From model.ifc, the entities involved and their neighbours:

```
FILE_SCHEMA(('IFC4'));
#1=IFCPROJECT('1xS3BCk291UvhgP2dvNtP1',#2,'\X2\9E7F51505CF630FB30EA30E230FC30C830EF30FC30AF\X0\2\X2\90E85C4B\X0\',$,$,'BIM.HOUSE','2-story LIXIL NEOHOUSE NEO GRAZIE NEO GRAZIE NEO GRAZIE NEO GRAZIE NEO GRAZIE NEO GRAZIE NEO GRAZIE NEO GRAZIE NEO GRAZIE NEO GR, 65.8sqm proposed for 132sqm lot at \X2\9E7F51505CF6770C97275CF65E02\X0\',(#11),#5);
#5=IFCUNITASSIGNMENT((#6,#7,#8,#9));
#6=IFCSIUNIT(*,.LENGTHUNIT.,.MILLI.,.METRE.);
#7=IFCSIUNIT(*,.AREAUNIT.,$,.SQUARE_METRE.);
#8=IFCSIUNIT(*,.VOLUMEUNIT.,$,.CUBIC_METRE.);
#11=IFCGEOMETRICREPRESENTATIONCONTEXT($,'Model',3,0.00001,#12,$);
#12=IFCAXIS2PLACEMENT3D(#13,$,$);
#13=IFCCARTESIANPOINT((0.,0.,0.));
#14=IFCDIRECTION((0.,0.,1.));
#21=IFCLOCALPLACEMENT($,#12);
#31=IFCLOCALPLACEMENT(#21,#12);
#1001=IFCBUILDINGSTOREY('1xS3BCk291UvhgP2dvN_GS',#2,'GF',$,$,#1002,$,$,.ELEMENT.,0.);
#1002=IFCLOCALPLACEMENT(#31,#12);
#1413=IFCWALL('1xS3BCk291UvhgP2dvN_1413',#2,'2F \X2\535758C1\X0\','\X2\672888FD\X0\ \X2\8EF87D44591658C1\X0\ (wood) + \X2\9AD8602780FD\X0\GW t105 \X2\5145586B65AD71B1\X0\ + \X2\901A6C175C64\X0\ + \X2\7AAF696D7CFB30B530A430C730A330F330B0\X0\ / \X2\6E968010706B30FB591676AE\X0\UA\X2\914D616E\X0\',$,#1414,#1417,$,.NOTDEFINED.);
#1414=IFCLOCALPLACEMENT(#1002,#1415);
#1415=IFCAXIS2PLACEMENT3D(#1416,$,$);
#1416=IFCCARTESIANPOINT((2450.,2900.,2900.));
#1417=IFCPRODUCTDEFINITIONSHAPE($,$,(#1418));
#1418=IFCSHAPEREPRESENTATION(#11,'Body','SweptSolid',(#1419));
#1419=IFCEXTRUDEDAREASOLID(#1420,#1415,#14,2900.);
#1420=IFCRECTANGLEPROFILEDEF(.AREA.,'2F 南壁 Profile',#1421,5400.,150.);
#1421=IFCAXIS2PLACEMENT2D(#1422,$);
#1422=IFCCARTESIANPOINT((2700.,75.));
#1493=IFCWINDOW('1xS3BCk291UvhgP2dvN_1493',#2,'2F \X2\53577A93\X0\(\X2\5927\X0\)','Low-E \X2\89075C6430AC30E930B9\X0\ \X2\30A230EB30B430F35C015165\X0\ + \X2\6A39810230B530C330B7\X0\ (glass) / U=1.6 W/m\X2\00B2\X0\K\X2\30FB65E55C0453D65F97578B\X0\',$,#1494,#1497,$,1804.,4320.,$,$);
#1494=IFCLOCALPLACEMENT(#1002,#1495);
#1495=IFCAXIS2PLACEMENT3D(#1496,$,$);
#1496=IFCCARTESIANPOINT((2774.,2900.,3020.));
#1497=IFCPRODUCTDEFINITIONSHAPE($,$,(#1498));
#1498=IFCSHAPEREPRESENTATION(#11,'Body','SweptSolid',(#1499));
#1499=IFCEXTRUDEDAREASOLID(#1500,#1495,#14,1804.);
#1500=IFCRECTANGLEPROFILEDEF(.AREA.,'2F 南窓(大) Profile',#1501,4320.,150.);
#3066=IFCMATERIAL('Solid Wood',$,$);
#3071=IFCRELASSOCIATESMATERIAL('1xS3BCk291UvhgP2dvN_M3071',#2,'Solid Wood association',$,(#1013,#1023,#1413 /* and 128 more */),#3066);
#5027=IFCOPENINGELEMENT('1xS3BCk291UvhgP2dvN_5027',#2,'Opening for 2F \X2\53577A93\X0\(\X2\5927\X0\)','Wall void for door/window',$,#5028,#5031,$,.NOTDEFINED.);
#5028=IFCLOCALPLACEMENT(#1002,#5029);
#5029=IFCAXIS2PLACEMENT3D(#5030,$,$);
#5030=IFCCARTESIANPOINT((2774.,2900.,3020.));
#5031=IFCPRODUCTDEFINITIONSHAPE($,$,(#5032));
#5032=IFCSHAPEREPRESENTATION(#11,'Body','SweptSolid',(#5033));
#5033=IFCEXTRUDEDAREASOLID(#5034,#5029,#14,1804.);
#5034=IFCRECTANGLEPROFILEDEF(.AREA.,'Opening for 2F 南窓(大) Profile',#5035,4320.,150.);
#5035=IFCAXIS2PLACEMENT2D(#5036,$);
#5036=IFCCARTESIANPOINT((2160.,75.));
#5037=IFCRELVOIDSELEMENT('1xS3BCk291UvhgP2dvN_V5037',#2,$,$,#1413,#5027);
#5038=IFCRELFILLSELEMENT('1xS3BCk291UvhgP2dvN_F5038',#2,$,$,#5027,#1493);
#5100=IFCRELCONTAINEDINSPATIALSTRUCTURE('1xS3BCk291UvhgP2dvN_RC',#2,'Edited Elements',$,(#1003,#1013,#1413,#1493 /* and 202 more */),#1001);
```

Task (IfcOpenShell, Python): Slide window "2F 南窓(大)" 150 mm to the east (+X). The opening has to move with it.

```python
import ifcopenshell
import ifcopenshell.api.geometry
import ifcopenshell.util.placement
import ifcopenshell.util.unit

model = ifcopenshell.open("model.ifc")
unit_scale = ifcopenshell.util.unit.calculate_unit_scale(model)

window = model.by_id(1493)
opening = window.FillsVoids[0].RelatingOpeningElement
wall = opening.VoidsElements[0].RelatingBuildingElement

wall_matrix = ifcopenshell.util.placement.get_local_placement(wall.ObjectPlacement)
shift = wall_matrix[:3, 0] * 0.15 / unit_scale
before = ifcopenshell.util.placement.get_local_placement(window.ObjectPlacement)[:3, 3].copy()

# The window is not placed relative to its opening, so move both.
for product in (opening, window):
    matrix = ifcopenshell.util.placement.get_local_placement(product.ObjectPlacement)
    matrix[:3, 3] += shift
    ifcopenshell.api.geometry.edit_object_placement(model, product=product, matrix=matrix, is_si=False)

after = ifcopenshell.util.placement.get_local_placement(window.ObjectPlacement)[:3, 3]
print("window moved by", (after - before).round(3) + 0.0)

model.write("model_updated.ifc")
```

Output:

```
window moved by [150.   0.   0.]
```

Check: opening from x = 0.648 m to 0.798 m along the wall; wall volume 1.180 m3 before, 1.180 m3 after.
